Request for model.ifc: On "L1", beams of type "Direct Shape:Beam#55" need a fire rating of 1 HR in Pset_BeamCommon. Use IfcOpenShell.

First a look at what the model holds.

```python
import ifcopenshell
import ifcopenshell.util.element

model = ifcopenshell.open("model.ifc")
print(model.schema)
storey = next(s for s in model.by_type("IfcBuildingStorey") if s.Name == "L1")
beams = [e for e in ifcopenshell.util.element.get_decomposition(storey) if e.is_a("IfcBeam")]
seen = {}
for e in beams:
    element_type = ifcopenshell.util.element.get_type(e)
    key = (element_type.Name if element_type != e and element_type else None, ifcopenshell.util.element.get_pset(e, "Pset_BeamCommon", "FireRating"))
    seen[key] = seen.get(key, 0) + 1
for (name, value), count in sorted(seen.items(), key=str):
    print(count, "x", name, "|", value)
```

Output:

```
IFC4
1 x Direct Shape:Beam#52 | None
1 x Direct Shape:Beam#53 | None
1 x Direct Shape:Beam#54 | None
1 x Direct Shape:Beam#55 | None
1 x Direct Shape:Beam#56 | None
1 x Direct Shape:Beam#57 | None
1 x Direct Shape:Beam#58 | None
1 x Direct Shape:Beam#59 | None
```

```python
import ifcopenshell
import ifcopenshell.api.pset
import ifcopenshell.util.element

model = ifcopenshell.open("model.ifc")

storey = next(s for s in model.by_type("IfcBuildingStorey") if s.Name == "L1")
beams = [e for e in ifcopenshell.util.element.get_decomposition(storey) if e.is_a("IfcBeam")]

count = 0
for e in beams:
    element_type = ifcopenshell.util.element.get_type(e)
    if element_type in (None, e) or element_type.Name != "Direct Shape:Beam#55":
        continue
    # add_pset returns the element's existing set when there is one.
    pset = ifcopenshell.api.pset.add_pset(model, product=e, name="Pset_BeamCommon")
    ifcopenshell.api.pset.edit_pset(model, pset=pset, properties={"FireRating": "1 HR"})
    count += 1

print(count, "beams updated")

model.write("model_rev.ifc")
```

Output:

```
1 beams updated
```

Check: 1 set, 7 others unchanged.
